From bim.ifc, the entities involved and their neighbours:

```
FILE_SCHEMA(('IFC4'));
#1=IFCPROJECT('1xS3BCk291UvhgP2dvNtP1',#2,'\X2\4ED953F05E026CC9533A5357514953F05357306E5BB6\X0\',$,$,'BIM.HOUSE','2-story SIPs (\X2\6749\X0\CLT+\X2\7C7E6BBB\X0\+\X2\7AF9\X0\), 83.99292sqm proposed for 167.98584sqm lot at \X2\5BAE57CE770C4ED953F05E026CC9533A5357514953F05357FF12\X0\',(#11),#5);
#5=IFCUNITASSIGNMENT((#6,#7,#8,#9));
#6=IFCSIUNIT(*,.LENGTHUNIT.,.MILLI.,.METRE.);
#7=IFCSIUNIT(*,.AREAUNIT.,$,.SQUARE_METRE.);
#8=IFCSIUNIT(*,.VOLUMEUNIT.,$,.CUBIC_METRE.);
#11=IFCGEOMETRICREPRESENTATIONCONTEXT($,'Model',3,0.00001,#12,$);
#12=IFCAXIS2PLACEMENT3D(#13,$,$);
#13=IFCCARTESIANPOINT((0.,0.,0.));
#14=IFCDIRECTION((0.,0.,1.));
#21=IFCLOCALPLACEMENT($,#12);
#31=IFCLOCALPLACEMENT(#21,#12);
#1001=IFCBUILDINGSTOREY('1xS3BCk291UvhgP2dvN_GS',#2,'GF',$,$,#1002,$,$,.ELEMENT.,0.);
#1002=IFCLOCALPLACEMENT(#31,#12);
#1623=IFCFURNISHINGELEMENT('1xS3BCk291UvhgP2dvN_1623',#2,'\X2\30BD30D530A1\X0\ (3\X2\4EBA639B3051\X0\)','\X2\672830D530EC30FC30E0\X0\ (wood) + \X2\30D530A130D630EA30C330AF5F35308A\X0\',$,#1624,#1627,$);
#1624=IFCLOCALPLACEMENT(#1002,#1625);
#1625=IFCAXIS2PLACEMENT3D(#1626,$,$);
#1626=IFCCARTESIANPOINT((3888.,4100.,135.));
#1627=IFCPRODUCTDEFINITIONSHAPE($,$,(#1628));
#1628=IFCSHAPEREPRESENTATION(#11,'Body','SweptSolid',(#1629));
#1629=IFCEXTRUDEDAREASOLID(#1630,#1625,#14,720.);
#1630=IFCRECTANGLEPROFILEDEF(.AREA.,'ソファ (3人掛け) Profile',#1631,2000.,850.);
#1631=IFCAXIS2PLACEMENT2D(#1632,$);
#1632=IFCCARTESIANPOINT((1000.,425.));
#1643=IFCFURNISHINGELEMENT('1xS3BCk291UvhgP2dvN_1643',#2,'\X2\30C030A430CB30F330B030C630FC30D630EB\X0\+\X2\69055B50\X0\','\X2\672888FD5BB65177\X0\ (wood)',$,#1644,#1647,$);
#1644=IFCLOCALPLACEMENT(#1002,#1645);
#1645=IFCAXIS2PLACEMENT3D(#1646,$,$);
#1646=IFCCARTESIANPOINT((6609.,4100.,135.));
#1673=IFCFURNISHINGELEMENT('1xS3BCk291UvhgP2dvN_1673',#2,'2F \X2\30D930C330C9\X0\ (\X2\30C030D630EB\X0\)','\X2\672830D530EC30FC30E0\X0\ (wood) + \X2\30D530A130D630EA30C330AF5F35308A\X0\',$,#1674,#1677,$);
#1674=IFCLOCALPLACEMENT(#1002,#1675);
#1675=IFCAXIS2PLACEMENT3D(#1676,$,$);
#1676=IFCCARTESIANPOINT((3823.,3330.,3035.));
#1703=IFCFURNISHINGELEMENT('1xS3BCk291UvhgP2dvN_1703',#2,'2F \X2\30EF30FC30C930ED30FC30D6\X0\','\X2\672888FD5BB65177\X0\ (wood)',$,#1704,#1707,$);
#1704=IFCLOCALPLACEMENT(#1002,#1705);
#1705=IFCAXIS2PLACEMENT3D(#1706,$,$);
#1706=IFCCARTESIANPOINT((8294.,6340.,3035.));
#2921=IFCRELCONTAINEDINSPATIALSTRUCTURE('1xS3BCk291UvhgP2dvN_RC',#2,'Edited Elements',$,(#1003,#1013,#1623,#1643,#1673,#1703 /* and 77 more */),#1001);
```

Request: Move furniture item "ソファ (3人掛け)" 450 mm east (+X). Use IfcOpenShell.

```python
import ifcopenshell
import ifcopenshell.api.geometry
import ifcopenshell.util.placement
import ifcopenshell.util.unit

model = ifcopenshell.open("bim.ifc")
unit_scale = ifcopenshell.util.unit.calculate_unit_scale(model)

item = model.by_id(1623)
matrix = ifcopenshell.util.placement.get_local_placement(item.ObjectPlacement)
matrix[0, 3] += 0.45 / unit_scale
ifcopenshell.api.geometry.edit_object_placement(model, product=item, matrix=matrix, is_si=False)

print(ifcopenshell.util.placement.get_local_placement(item.ObjectPlacement).round(3) + 0.0)

model.write("bim_v2.ifc")
```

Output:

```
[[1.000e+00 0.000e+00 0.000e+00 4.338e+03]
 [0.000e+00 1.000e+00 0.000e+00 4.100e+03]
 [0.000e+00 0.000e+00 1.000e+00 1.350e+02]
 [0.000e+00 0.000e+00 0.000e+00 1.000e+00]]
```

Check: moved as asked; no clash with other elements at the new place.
